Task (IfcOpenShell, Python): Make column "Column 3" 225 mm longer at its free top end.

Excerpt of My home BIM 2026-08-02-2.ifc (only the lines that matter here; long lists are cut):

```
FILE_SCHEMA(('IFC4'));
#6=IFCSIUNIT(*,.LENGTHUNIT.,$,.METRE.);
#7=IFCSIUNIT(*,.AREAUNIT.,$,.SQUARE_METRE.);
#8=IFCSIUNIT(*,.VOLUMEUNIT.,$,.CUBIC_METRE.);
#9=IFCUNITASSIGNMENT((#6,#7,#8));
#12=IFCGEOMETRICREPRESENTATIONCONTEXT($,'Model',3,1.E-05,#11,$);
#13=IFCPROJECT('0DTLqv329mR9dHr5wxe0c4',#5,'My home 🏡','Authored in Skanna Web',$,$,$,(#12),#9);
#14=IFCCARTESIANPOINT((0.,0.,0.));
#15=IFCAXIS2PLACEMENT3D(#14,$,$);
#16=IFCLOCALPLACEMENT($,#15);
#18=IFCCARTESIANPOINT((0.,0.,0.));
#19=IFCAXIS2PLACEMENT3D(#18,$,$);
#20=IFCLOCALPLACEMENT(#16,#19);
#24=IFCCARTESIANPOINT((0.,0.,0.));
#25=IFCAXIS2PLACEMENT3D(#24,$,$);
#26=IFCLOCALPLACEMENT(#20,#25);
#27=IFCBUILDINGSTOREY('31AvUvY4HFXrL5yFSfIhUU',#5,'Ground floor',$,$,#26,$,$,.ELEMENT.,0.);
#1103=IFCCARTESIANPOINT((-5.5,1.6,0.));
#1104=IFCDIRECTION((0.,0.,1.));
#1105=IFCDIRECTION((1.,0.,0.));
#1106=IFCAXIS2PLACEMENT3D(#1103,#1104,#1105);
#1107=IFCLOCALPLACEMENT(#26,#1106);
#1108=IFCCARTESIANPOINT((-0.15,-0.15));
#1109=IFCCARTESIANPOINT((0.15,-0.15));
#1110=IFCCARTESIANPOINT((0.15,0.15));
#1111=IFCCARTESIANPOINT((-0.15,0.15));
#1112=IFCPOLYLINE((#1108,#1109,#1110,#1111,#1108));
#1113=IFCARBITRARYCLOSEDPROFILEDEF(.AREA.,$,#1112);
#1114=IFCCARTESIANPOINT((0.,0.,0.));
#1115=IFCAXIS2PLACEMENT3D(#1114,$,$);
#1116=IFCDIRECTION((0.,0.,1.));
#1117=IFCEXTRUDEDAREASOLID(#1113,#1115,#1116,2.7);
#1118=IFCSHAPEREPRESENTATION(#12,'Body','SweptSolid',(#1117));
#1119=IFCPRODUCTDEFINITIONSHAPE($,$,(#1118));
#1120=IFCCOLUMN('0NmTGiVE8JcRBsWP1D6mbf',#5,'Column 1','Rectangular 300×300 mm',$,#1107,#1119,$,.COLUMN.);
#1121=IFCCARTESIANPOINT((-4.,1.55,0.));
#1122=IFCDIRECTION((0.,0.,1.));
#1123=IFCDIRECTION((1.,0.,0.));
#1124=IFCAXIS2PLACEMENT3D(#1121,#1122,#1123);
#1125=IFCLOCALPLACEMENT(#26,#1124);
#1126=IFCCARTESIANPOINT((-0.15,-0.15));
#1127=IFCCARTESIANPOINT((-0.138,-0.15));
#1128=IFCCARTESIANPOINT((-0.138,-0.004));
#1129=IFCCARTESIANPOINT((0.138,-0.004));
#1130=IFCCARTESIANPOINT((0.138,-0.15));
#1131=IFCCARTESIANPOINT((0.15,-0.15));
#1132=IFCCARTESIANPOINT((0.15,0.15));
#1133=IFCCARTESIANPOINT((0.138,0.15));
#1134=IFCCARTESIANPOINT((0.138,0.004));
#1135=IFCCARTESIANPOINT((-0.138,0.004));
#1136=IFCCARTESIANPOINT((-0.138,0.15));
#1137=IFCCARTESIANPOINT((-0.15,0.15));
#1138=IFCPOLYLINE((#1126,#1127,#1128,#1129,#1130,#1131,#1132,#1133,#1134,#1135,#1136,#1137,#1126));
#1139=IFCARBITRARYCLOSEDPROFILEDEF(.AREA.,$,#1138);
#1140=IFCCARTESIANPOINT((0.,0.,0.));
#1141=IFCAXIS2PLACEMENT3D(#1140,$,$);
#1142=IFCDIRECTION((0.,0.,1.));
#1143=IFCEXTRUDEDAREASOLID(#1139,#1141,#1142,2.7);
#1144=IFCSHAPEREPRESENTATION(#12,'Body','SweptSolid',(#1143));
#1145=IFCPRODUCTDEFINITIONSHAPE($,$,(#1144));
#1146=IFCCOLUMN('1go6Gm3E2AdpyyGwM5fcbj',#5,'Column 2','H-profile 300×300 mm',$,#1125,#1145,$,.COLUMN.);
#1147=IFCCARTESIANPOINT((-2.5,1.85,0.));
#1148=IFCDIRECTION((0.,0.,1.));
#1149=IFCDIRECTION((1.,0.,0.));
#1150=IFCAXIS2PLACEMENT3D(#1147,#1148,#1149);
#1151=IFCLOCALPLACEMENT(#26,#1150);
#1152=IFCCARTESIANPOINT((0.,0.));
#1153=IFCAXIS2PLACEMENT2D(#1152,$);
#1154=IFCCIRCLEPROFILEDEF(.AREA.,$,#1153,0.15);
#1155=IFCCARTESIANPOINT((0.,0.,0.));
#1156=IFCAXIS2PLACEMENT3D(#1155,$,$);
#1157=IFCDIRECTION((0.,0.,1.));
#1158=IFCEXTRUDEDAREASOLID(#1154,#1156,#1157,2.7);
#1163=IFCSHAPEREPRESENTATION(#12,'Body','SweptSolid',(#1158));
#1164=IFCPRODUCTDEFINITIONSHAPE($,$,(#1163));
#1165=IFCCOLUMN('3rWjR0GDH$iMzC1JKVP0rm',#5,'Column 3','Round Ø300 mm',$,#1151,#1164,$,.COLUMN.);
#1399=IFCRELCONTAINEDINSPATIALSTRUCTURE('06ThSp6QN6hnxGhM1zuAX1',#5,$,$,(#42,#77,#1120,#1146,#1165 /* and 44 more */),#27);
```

```python
import ifcopenshell
import ifcopenshell.util.unit

model = ifcopenshell.open("My home BIM 2026-08-02-2.ifc")
unit_scale = ifcopenshell.util.unit.calculate_unit_scale(model)

member = model.by_guid("3rWjR0GDH$iMzC1JKVP0rm")
change = 0.225 / unit_scale

# The extrusion runs towards the end named, so only its depth changes.
body = next(r for r in member.Representation.Representations if r.RepresentationIdentifier == "Body")
solid = body.Items[0]
old_length = solid.Depth
solid.Depth += change

print(f"length {old_length:g} -> {solid.Depth:g}")

model.write("My home BIM 2026-08-02-2_edited.ifc")
```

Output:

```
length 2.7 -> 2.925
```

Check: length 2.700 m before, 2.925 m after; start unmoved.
